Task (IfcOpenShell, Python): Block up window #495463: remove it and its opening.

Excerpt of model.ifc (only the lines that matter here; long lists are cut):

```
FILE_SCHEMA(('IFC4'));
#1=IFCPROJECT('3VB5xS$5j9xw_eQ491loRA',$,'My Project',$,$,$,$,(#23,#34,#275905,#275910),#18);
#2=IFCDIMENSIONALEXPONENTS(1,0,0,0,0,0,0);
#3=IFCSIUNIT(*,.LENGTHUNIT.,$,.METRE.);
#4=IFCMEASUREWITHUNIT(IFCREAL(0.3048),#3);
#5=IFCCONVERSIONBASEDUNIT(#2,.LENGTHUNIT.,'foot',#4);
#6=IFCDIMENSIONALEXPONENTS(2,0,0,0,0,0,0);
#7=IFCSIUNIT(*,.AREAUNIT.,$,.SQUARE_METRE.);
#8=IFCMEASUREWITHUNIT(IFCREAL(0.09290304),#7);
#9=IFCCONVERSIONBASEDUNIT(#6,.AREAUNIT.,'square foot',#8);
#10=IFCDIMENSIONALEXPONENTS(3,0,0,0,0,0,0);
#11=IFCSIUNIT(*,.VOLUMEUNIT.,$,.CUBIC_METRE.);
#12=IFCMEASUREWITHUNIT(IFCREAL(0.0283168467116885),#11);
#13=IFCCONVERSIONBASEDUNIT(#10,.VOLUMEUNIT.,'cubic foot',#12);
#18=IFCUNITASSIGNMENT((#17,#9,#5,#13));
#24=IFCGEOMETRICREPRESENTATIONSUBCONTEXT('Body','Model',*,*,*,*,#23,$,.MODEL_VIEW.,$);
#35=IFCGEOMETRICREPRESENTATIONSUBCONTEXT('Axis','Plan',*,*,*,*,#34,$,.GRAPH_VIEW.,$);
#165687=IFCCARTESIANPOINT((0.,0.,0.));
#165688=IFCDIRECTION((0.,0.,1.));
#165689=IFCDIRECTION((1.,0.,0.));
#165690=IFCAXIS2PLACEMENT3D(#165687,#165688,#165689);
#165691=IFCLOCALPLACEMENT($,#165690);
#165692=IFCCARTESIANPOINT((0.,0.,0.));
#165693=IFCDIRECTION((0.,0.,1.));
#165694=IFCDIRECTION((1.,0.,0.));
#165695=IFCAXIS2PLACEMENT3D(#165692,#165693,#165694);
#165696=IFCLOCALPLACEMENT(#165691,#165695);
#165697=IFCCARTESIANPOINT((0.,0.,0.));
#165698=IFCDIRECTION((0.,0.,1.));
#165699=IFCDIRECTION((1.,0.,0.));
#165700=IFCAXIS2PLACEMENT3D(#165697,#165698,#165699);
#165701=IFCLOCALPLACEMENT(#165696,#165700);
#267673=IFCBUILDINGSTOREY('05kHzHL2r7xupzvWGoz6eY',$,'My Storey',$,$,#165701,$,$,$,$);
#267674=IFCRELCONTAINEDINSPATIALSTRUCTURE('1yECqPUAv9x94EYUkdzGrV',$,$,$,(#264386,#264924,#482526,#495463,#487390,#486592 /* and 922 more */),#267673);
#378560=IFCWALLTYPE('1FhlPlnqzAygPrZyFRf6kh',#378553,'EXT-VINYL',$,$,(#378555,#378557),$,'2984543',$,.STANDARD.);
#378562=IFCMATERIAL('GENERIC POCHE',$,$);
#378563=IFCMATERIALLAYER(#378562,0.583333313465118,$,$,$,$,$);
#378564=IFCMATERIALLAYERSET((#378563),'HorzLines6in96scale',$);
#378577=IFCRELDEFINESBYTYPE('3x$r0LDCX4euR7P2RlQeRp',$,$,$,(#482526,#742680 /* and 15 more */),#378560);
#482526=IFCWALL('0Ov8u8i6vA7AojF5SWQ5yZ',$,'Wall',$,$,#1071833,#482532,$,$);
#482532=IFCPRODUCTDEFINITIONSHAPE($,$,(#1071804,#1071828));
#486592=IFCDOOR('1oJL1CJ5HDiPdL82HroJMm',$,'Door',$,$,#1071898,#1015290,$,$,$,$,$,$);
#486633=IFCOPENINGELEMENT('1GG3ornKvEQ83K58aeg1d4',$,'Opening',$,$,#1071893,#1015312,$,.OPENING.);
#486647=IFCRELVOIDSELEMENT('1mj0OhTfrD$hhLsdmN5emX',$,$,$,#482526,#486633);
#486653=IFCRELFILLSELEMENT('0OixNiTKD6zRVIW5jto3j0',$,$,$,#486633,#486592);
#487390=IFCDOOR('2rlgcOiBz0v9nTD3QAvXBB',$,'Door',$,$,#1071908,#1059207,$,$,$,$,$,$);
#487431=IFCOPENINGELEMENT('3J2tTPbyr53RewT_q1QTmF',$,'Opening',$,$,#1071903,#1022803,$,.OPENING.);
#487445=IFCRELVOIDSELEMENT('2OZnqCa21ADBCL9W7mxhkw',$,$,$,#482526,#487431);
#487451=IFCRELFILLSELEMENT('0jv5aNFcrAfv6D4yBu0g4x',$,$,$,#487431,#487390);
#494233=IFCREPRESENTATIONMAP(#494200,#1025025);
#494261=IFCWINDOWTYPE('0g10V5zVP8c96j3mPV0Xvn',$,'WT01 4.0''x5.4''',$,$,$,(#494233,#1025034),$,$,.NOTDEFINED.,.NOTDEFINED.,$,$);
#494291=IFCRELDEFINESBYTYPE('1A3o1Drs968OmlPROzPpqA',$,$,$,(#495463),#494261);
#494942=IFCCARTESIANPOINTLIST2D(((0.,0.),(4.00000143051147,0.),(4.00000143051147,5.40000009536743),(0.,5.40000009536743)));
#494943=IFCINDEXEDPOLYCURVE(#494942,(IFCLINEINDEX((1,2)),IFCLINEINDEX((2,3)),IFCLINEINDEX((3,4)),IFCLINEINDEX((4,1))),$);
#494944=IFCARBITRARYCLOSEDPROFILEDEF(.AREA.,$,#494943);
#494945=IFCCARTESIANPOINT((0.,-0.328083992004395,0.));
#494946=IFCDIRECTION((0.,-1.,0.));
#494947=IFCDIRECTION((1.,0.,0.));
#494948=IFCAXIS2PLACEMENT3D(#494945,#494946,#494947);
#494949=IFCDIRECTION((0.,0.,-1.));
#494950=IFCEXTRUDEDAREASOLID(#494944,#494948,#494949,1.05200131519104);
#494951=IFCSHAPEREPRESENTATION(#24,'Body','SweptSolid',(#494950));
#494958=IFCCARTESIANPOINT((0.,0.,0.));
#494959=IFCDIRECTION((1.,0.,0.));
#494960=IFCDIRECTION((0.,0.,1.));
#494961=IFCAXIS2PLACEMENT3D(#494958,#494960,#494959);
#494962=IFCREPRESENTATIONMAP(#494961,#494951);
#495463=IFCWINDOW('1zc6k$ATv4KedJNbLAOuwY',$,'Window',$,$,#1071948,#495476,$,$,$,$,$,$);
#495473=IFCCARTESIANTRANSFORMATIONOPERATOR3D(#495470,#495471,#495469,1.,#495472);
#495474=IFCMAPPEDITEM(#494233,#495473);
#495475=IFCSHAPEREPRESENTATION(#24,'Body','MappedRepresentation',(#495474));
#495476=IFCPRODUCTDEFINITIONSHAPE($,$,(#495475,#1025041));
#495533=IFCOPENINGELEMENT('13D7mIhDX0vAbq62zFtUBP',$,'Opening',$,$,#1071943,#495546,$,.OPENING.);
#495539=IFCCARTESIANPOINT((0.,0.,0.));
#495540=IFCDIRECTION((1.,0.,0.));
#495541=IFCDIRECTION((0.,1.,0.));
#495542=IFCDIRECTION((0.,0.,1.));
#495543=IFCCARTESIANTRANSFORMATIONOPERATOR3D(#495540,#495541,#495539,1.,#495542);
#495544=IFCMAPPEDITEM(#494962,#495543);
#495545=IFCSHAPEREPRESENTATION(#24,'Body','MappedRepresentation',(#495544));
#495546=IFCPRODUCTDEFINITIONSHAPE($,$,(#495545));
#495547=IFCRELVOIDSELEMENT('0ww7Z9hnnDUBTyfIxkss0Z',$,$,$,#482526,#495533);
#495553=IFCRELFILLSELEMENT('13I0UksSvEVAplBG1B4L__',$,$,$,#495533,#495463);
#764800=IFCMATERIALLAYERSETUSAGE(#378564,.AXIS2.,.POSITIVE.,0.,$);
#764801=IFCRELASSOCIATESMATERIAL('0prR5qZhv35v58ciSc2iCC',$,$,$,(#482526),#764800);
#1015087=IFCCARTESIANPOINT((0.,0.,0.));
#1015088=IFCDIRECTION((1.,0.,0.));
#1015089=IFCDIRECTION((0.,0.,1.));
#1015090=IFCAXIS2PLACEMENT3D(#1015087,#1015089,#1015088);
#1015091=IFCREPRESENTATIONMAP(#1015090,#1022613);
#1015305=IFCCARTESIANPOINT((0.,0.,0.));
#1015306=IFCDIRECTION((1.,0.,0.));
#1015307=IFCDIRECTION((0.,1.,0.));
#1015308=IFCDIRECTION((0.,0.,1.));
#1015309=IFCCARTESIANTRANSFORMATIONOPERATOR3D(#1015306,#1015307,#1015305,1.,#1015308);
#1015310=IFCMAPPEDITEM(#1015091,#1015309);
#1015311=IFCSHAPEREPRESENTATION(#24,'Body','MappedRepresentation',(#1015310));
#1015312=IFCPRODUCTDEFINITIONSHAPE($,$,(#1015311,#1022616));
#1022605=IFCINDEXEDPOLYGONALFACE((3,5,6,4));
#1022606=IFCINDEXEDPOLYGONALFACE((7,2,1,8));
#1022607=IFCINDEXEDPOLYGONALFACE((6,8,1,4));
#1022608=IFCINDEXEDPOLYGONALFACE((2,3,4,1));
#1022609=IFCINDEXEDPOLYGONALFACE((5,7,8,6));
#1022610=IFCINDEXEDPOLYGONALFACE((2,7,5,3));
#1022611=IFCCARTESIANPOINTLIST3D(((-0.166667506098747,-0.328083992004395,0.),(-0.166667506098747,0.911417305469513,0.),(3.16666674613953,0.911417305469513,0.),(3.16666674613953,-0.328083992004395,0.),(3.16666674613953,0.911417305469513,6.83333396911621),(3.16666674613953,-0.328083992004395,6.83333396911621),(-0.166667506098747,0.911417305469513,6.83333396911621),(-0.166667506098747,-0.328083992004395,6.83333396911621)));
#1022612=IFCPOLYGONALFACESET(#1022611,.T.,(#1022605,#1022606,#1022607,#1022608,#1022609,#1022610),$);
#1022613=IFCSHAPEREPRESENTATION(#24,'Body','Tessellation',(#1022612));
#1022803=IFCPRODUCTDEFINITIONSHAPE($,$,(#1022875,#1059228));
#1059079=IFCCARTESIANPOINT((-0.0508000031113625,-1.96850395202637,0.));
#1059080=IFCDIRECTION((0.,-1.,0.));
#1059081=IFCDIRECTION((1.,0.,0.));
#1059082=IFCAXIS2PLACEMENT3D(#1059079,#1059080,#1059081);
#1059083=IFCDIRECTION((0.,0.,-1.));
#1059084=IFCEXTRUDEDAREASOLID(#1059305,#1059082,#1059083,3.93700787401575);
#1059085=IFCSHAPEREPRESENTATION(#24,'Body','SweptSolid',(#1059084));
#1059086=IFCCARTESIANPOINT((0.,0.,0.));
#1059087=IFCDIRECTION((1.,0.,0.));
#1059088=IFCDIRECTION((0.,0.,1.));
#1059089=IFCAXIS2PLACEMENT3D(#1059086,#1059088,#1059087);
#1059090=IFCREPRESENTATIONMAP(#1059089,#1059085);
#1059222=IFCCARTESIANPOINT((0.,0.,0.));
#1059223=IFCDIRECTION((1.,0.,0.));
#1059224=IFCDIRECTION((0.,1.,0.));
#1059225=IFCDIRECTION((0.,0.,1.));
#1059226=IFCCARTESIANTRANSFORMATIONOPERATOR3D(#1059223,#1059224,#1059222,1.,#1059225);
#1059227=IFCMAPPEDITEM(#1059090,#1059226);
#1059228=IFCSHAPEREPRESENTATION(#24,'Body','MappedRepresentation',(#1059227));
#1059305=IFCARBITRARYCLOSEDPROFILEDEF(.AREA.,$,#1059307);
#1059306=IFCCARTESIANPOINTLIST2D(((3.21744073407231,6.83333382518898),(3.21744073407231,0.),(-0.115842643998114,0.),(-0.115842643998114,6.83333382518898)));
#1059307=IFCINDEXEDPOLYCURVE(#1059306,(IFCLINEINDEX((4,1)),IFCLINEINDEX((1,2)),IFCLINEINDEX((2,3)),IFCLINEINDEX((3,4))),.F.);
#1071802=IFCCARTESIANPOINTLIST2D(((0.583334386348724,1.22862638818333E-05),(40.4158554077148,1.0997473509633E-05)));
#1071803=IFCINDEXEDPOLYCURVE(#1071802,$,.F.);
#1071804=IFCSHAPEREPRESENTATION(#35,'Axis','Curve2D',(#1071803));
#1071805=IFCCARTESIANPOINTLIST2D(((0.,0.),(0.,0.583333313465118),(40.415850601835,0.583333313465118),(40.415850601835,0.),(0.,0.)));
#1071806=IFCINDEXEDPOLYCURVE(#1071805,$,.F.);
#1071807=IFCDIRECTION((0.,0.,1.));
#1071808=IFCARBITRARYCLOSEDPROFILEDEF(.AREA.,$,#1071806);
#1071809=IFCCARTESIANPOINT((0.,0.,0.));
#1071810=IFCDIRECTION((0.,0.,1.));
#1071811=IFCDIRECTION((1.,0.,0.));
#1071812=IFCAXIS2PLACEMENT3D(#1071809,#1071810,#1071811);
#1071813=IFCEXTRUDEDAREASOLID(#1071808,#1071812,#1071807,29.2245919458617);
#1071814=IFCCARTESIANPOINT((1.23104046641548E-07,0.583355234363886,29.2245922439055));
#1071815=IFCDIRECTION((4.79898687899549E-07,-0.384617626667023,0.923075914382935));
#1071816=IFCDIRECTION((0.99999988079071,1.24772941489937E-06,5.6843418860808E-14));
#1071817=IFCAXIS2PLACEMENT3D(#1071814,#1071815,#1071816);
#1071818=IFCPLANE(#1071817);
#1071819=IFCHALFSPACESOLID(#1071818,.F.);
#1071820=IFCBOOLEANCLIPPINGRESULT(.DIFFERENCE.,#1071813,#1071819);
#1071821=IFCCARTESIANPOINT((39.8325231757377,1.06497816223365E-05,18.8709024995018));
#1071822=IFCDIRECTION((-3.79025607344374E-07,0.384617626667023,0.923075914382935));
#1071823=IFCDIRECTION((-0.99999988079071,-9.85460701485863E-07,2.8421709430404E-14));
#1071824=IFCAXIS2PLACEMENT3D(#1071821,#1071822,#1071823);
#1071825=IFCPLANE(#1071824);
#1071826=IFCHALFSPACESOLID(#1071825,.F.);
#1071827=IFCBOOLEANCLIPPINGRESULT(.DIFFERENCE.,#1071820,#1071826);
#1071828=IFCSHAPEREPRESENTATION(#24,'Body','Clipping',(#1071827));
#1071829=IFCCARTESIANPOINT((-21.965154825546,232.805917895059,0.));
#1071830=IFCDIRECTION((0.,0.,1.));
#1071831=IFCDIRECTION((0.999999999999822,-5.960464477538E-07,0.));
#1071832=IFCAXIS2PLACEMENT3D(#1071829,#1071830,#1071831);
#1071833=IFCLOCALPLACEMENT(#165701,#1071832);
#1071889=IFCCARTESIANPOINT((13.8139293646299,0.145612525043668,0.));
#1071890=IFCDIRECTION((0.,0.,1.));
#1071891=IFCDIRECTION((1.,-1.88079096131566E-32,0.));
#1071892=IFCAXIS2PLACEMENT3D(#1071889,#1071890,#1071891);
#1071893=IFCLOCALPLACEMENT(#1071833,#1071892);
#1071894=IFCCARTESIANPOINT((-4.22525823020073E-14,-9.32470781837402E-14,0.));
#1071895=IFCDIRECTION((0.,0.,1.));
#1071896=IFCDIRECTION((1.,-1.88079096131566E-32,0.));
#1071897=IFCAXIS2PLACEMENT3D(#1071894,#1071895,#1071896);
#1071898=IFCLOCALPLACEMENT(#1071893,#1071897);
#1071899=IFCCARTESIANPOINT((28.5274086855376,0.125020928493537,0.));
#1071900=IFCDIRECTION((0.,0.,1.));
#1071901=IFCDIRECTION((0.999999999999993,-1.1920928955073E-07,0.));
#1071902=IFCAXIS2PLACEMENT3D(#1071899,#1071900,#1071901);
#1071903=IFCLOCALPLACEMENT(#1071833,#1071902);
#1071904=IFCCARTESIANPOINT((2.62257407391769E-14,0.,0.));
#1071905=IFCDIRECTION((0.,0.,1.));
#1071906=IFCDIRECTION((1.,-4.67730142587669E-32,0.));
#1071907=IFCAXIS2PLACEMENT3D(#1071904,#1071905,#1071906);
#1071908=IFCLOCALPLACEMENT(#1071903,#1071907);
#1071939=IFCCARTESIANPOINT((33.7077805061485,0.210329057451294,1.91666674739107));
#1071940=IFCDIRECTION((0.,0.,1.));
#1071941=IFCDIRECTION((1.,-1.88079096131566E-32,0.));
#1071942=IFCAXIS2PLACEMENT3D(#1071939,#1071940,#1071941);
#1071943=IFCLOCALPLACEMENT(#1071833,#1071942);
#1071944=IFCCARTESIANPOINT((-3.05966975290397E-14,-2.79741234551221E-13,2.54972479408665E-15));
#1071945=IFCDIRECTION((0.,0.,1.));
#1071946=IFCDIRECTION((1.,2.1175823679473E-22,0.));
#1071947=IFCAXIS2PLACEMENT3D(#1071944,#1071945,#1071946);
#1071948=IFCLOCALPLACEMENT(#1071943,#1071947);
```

```python
import ifcopenshell
import ifcopenshell.api.feature
import ifcopenshell.api.root
import ifcopenshell.geom
import ifcopenshell.util.shape

model = ifcopenshell.open("model.ifc")
settings = ifcopenshell.geom.settings()


def volume(element):
    """Net volume in cubic metres, openings subtracted."""
    shape = ifcopenshell.geom.create_shape(settings, element)
    return ifcopenshell.util.shape.get_volume(shape.geometry)


window = model.by_guid("1zc6k$ATv4KedJNbLAOuwY")
opening = window.FillsVoids[0].RelatingOpeningElement
wall = opening.VoidsElements[0].RelatingBuildingElement
before = volume(wall)

ifcopenshell.api.root.remove_product(model, product=window)
ifcopenshell.api.feature.remove_feature(model, feature=opening)

after = volume(wall)

print(f"wall volume {before:.3f} -> {after:.3f} m3")

model.write("model-out.ifc")
```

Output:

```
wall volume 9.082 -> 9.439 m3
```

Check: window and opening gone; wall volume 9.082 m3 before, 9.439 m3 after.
